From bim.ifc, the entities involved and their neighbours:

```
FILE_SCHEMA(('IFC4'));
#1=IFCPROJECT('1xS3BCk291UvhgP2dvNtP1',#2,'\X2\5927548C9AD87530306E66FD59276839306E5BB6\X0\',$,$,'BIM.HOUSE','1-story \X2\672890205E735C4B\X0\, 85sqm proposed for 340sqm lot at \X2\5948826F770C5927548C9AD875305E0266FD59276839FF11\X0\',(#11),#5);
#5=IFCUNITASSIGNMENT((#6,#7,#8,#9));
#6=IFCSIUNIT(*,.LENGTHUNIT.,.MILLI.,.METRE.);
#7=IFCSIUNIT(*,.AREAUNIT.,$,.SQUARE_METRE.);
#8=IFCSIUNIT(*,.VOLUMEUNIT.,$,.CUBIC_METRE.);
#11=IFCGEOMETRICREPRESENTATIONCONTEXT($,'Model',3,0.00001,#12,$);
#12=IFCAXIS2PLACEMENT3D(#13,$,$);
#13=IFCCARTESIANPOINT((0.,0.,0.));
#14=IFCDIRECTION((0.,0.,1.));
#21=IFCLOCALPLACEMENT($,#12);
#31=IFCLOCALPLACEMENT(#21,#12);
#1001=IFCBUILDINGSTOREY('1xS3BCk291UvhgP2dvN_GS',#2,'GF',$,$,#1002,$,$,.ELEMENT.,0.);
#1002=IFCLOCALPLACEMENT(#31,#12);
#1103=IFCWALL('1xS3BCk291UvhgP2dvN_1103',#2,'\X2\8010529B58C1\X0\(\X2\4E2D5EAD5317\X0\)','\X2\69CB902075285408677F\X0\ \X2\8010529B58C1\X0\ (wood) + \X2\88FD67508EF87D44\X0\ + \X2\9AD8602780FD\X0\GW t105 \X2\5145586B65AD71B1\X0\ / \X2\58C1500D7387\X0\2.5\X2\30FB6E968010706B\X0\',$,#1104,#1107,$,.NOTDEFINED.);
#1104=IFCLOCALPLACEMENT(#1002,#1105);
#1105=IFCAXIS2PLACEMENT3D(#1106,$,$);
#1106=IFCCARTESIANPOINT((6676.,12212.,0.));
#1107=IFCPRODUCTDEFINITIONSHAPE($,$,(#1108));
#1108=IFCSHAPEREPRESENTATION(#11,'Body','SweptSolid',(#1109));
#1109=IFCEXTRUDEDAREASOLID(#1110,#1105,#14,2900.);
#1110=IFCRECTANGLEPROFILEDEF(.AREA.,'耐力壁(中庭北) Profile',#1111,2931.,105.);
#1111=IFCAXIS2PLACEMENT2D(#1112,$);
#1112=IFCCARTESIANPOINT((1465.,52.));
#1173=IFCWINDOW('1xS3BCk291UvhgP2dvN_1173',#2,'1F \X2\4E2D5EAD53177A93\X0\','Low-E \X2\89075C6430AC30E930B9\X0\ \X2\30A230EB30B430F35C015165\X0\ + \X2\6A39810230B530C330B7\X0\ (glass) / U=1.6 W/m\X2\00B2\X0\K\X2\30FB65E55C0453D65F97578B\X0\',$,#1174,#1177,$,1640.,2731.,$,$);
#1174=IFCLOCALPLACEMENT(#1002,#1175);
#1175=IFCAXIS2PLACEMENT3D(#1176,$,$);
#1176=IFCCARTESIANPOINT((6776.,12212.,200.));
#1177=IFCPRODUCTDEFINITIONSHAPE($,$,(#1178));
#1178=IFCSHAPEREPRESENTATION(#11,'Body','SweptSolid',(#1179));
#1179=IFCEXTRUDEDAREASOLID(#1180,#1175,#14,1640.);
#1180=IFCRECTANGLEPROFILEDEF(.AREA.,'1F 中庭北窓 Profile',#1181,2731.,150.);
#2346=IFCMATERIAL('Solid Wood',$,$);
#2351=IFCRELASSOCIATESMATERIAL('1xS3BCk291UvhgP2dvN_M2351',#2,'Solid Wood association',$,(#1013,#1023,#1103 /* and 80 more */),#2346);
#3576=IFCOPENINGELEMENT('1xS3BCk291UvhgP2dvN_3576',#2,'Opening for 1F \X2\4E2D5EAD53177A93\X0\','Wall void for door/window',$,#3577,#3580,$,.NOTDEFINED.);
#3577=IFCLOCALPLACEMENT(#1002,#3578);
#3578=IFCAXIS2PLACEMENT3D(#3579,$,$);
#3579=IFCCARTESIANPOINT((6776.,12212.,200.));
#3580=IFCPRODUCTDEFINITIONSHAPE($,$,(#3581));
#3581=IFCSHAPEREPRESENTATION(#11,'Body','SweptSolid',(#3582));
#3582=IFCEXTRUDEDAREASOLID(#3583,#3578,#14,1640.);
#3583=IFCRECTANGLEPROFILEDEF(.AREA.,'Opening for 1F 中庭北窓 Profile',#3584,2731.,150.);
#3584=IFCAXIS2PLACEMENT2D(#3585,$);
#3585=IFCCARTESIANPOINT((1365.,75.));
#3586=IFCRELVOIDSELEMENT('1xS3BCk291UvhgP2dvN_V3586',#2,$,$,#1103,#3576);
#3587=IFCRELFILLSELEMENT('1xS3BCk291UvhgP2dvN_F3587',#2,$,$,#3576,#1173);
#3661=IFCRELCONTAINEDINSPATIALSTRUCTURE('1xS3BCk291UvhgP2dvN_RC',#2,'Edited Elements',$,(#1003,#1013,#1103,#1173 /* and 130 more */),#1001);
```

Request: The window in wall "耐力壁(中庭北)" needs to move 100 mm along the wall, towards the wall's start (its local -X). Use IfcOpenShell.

```python
import ifcopenshell
import ifcopenshell.api.geometry
import ifcopenshell.util.placement

model = ifcopenshell.open("bim.ifc")

window = model.by_id(1173)
opening = window.FillsVoids[0].RelatingOpeningElement
wall = opening.VoidsElements[0].RelatingBuildingElement

wall_matrix = ifcopenshell.util.placement.get_local_placement(wall.ObjectPlacement)
shift = wall_matrix[:3, 0] * -100.0
before = ifcopenshell.util.placement.get_local_placement(window.ObjectPlacement)[:3, 3].copy()

# The window is not placed relative to its opening, so move both.
for product in (opening, window):
    matrix = ifcopenshell.util.placement.get_local_placement(product.ObjectPlacement)
    matrix[:3, 3] += shift
    ifcopenshell.api.geometry.edit_object_placement(model, product=product, matrix=matrix, is_si=False)

after = ifcopenshell.util.placement.get_local_placement(window.ObjectPlacement)[:3, 3]
print("window moved by", (after - before).round(3) + 0.0)

model.write("bim_v2.ifc")
```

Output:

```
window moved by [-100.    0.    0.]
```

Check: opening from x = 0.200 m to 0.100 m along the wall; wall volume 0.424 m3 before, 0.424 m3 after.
